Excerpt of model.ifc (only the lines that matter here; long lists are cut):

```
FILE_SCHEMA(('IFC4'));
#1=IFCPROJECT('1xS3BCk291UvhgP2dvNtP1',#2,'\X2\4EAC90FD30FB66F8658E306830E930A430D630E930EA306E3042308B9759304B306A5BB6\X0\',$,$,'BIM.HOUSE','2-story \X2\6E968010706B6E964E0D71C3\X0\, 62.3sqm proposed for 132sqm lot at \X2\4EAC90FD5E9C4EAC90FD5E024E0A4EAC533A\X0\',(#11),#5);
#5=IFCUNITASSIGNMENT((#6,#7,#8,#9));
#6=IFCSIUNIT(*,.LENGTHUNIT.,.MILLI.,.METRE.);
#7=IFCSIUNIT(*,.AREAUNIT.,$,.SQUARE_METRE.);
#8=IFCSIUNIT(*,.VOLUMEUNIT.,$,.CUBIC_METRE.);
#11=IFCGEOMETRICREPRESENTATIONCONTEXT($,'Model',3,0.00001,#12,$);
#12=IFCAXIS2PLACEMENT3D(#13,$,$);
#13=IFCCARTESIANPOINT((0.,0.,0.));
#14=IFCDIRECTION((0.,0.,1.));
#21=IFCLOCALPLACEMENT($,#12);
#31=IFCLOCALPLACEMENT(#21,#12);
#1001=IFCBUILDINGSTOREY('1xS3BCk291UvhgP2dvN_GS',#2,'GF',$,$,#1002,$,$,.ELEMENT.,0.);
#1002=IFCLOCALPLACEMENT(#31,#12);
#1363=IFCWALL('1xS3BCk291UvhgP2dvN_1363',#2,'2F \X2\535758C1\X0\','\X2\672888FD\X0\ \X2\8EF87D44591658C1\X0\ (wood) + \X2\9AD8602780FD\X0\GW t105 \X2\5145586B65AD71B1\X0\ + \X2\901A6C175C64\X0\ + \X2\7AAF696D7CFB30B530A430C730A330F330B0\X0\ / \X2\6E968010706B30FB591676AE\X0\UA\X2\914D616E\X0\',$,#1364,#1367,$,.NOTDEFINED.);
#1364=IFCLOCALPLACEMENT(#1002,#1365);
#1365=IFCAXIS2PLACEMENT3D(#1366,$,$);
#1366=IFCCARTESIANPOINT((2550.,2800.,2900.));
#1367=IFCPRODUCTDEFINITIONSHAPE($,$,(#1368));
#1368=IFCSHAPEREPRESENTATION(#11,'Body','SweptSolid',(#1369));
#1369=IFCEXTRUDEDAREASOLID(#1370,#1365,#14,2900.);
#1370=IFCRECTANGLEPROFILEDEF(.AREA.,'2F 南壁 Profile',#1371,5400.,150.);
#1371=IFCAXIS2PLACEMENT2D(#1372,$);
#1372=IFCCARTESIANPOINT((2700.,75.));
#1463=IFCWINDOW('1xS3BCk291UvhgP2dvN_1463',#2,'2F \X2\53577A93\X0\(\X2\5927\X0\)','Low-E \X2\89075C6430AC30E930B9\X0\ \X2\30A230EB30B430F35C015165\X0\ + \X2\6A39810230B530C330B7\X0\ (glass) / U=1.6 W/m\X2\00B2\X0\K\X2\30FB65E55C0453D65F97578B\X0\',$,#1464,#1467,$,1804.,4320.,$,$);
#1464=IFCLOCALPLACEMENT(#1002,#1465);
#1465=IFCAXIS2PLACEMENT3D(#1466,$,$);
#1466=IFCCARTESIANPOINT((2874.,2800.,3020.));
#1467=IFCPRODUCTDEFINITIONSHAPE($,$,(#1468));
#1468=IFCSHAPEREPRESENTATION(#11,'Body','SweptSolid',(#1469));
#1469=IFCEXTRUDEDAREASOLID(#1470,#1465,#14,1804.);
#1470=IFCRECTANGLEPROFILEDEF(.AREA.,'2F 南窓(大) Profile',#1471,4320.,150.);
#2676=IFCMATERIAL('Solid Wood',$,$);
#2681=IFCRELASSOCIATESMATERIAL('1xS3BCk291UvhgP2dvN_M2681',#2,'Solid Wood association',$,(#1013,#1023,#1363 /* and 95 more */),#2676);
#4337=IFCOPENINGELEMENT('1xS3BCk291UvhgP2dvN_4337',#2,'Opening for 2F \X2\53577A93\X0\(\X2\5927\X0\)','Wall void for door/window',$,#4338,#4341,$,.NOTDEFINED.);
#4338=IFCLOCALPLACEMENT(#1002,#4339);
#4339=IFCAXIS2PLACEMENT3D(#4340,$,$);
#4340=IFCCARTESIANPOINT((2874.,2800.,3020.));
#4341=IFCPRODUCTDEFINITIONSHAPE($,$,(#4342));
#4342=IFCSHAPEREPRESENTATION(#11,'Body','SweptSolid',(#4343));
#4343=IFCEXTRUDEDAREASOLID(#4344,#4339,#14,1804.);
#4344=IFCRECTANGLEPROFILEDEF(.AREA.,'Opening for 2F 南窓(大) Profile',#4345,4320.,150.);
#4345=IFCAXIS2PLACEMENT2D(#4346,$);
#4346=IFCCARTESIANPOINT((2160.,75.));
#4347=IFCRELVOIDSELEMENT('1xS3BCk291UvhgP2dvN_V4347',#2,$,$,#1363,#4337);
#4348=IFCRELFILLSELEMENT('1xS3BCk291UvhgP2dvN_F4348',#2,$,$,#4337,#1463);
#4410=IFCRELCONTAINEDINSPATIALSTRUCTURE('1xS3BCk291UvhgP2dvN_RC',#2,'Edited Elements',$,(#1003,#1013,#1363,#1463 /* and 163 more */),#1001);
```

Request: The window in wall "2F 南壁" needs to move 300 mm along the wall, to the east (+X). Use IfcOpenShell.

```python
import ifcopenshell
import ifcopenshell.api.geometry
import ifcopenshell.util.placement
import ifcopenshell.util.unit

model = ifcopenshell.open("model.ifc")
unit_scale = ifcopenshell.util.unit.calculate_unit_scale(model)

window = model.by_id(1463)
opening = window.FillsVoids[0].RelatingOpeningElement
wall = opening.VoidsElements[0].RelatingBuildingElement

wall_matrix = ifcopenshell.util.placement.get_local_placement(wall.ObjectPlacement)
shift = wall_matrix[:3, 0] * 0.3 / unit_scale
before = ifcopenshell.util.placement.get_local_placement(window.ObjectPlacement)[:3, 3].copy()

# The window is not placed relative to its opening, so move both.
for product in (opening, window):
    matrix = ifcopenshell.util.placement.get_local_placement(product.ObjectPlacement)
    matrix[:3, 3] += shift
    ifcopenshell.api.geometry.edit_object_placement(model, product=product, matrix=matrix, is_si=False)

after = ifcopenshell.util.placement.get_local_placement(window.ObjectPlacement)[:3, 3]
print("window moved by", (after - before).round(3) + 0.0)

model.write("model-out.ifc")
```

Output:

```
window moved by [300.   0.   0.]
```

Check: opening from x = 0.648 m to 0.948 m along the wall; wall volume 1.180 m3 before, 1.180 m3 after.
